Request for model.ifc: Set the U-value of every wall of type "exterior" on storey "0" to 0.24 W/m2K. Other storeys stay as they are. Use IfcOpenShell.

First a look at what the model holds.

```python
import ifcopenshell
import ifcopenshell.util.element

model = ifcopenshell.open("model.ifc")
print(model.schema)
storey = next(s for s in model.by_type("IfcBuildingStorey") if s.Name == "0")
walls = [e for e in ifcopenshell.util.element.get_decomposition(storey) if e.is_a("IfcWall")]
seen = {}
for e in walls:
    element_type = ifcopenshell.util.element.get_type(e)
    key = (element_type.Name if element_type != e and element_type else None, ifcopenshell.util.element.get_pset(e, "Pset_WallCommon", "ThermalTransmittance"))
    seen[key] = seen.get(key, 0) + 1
for (name, value), count in sorted(seen.items(), key=str):
    print(count, "x", name, "|", value)
```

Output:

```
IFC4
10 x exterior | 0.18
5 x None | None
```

```python
import ifcopenshell
import ifcopenshell.api.pset
import ifcopenshell.util.element

model = ifcopenshell.open("model.ifc")

storey = next(s for s in model.by_type("IfcBuildingStorey") if s.Name == "0")
walls = [e for e in ifcopenshell.util.element.get_decomposition(storey) if e.is_a("IfcWall")]

count = 0
for e in walls:
    element_type = ifcopenshell.util.element.get_type(e)
    if element_type in (None, e) or element_type.Name != "exterior":
        continue
    # add_pset returns the element's existing set when there is one.
    pset = ifcopenshell.api.pset.add_pset(model, product=e, name="Pset_WallCommon")
    ifcopenshell.api.pset.edit_pset(model, pset=pset, properties={"ThermalTransmittance": 0.24})
    count += 1

print(count, "walls updated")

model.write("model_updated.ifc")
```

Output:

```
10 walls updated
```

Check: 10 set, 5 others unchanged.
